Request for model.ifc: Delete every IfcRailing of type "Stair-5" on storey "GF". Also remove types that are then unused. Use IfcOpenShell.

First a look at what the model holds.

```python
import ifcopenshell
import ifcopenshell.util.element

model = ifcopenshell.open("model.ifc")
print(model.schema)
storey = next(s for s in model.by_type("IfcBuildingStorey") if s.Name == "GF")
railings = [e for e in ifcopenshell.util.element.get_decomposition(storey) if e.is_a("IfcRailing")]
seen = {}
for e in railings:
    element_type = ifcopenshell.util.element.get_type(e)
    name = element_type.Name if element_type not in (None, e) else None
    seen[name] = seen.get(name, 0) + 1
for name, count in sorted(seen.items(), key=str):
    print(count, "x", name)
```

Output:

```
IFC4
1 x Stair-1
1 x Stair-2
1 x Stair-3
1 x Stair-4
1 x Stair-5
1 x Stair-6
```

```python
import ifcopenshell
import ifcopenshell.api.root
import ifcopenshell.util.element

model = ifcopenshell.open("model.ifc")

storey = next(s for s in model.by_type("IfcBuildingStorey") if s.Name == "GF")
railings = [e for e in ifcopenshell.util.element.get_decomposition(storey) if e.is_a("IfcRailing")]
targets = [e for e in railings if (t := ifcopenshell.util.element.get_type(e)) not in (None, e) and t.Name == "Stair-5"]
types = {ifcopenshell.util.element.get_type(e) for e in targets} - {None, *targets}

for e in targets:
    ifcopenshell.api.root.remove_product(model, product=e)
print(len(targets), "removed")

unused = [t for t in types if not ifcopenshell.util.element.get_types(t)]
for t in unused:
    ifcopenshell.api.root.remove_product(model, product=t)
print(len(unused), "unused types removed")

model.write("model_updated.ifc")
```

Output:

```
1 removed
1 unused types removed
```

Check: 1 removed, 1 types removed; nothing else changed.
